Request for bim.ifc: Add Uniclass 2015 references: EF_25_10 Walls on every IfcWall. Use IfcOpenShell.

First a look at what the model holds.

```python
import ifcopenshell

model = ifcopenshell.open("bim.ifc")
print(model.schema)
print("classifications:", [c.Name for c in model.by_type("IfcClassification")])
for ifc_class in ("IfcDoor", "IfcRoof", "IfcStair", "IfcWall", "IfcWindow"):
    print(ifc_class, len(model.by_type(ifc_class)))
```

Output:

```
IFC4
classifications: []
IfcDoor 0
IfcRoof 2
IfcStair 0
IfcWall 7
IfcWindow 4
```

```python
import ifcopenshell
import ifcopenshell.api.classification

model = ifcopenshell.open("bim.ifc")

system = ifcopenshell.api.classification.add_classification(model, classification="Uniclass 2015")

codes = {
    "IfcWall": ("EF_25_10", "Walls"),
}
for ifc_class, (code, name) in codes.items():
    products = model.by_type(ifc_class)
    ifcopenshell.api.classification.add_reference(
        model, products=products, classification=system, identification=code, name=name
    )
    print(code, len(products))

model.write("bim-out.ifc")
```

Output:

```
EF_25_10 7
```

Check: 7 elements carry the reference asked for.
